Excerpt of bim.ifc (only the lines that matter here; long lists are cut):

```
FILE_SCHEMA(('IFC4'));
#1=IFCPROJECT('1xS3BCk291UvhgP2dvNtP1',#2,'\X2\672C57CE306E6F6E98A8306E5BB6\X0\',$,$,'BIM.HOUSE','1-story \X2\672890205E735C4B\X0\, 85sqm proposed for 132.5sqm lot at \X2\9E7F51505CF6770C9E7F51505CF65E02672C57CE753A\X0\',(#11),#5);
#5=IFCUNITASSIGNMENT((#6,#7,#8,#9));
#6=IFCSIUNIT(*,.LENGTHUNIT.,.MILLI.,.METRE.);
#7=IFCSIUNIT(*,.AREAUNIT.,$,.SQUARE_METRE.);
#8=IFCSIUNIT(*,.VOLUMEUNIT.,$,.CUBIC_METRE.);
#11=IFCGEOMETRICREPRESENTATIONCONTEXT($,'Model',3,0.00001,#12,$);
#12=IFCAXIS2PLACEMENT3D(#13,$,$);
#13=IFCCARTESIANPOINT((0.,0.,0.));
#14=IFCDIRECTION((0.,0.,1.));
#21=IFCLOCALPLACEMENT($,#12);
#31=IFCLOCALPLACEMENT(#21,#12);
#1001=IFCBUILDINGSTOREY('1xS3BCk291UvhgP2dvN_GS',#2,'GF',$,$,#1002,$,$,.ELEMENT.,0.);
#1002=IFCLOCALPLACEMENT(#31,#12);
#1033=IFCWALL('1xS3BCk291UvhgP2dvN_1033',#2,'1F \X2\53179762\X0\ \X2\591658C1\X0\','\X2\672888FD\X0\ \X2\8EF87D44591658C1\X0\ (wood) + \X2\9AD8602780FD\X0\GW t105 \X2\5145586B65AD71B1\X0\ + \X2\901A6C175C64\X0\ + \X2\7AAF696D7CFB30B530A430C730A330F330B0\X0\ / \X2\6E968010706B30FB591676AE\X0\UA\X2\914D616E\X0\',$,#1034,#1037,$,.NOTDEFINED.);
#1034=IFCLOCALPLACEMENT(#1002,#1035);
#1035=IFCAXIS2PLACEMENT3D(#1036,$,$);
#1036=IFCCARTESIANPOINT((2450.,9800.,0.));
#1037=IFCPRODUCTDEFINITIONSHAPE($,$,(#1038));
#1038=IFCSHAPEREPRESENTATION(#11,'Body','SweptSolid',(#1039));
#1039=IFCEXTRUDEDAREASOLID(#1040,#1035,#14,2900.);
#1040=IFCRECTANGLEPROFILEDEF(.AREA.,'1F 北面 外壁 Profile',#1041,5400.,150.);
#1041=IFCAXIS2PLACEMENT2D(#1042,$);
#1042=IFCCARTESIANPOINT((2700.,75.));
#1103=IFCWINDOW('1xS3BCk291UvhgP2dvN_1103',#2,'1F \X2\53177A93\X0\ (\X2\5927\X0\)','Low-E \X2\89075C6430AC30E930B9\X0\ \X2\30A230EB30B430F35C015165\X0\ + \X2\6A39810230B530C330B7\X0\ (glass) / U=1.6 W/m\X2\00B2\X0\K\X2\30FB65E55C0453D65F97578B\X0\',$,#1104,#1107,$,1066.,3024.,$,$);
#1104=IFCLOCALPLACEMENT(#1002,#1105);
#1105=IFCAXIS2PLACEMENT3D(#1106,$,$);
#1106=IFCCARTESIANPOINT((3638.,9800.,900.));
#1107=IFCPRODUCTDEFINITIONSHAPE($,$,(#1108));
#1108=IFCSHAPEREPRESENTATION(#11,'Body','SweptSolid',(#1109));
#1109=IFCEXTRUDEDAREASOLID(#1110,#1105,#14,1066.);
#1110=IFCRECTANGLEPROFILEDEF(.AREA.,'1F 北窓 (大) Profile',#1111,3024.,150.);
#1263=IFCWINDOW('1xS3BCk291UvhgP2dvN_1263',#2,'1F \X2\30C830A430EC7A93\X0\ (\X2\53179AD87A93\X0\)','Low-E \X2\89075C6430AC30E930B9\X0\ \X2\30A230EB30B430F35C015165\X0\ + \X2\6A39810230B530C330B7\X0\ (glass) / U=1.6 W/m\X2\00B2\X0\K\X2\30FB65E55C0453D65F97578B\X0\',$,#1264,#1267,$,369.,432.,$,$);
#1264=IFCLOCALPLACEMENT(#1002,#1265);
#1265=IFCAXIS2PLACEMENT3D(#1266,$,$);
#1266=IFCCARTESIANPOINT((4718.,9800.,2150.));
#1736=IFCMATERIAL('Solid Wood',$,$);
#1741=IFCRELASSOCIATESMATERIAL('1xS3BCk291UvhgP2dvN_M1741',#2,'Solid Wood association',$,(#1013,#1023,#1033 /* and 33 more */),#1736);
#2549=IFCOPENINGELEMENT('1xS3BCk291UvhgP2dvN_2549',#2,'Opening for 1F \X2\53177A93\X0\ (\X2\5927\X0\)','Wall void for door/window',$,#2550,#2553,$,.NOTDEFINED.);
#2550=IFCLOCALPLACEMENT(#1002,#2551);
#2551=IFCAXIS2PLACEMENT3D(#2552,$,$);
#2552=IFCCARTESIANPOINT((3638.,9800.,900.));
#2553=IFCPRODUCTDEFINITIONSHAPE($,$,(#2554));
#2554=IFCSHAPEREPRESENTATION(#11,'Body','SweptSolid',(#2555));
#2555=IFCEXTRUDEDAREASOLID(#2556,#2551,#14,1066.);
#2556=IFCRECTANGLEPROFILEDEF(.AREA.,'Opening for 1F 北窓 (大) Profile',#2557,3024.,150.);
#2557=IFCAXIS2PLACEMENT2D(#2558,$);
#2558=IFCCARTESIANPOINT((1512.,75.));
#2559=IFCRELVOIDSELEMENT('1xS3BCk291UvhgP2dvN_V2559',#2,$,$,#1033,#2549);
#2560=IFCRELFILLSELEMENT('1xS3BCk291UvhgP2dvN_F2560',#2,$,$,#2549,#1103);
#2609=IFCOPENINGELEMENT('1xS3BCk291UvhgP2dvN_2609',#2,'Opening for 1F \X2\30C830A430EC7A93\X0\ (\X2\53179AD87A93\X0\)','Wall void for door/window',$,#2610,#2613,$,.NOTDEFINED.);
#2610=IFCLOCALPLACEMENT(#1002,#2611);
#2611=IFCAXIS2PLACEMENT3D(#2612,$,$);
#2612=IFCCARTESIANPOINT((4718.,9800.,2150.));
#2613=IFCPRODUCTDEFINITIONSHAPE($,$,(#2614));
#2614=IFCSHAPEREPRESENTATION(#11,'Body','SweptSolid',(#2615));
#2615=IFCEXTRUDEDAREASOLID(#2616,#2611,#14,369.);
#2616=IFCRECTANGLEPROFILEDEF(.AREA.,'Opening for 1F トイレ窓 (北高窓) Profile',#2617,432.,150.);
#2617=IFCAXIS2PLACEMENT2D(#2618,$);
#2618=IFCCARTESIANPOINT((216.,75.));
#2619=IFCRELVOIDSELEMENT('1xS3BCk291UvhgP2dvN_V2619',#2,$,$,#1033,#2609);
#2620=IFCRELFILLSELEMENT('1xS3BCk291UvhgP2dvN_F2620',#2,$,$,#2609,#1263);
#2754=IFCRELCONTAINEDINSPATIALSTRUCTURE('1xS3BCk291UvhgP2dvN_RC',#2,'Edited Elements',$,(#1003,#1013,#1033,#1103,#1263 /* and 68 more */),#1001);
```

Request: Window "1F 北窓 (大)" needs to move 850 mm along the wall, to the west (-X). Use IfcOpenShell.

```python
import ifcopenshell
import ifcopenshell.api.geometry
import ifcopenshell.util.placement
import ifcopenshell.util.unit

model = ifcopenshell.open("bim.ifc")
unit_scale = ifcopenshell.util.unit.calculate_unit_scale(model)

window = model.by_id(1103)
opening = window.FillsVoids[0].RelatingOpeningElement
wall = opening.VoidsElements[0].RelatingBuildingElement

wall_matrix = ifcopenshell.util.placement.get_local_placement(wall.ObjectPlacement)
shift = wall_matrix[:3, 0] * -0.85 / unit_scale
before = ifcopenshell.util.placement.get_local_placement(window.ObjectPlacement)[:3, 3].copy()

# The window is not placed relative to its opening, so move both.
for product in (opening, window):
    matrix = ifcopenshell.util.placement.get_local_placement(product.ObjectPlacement)
    matrix[:3, 3] += shift
    ifcopenshell.api.geometry.edit_object_placement(model, product=product, matrix=matrix, is_si=False)

after = ifcopenshell.util.placement.get_local_placement(window.ObjectPlacement)[:3, 3]
print("window moved by", (after - before).round(3) + 0.0)

model.write("bim_rev.ifc")
```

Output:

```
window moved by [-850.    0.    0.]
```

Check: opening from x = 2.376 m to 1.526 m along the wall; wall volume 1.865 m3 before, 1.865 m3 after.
